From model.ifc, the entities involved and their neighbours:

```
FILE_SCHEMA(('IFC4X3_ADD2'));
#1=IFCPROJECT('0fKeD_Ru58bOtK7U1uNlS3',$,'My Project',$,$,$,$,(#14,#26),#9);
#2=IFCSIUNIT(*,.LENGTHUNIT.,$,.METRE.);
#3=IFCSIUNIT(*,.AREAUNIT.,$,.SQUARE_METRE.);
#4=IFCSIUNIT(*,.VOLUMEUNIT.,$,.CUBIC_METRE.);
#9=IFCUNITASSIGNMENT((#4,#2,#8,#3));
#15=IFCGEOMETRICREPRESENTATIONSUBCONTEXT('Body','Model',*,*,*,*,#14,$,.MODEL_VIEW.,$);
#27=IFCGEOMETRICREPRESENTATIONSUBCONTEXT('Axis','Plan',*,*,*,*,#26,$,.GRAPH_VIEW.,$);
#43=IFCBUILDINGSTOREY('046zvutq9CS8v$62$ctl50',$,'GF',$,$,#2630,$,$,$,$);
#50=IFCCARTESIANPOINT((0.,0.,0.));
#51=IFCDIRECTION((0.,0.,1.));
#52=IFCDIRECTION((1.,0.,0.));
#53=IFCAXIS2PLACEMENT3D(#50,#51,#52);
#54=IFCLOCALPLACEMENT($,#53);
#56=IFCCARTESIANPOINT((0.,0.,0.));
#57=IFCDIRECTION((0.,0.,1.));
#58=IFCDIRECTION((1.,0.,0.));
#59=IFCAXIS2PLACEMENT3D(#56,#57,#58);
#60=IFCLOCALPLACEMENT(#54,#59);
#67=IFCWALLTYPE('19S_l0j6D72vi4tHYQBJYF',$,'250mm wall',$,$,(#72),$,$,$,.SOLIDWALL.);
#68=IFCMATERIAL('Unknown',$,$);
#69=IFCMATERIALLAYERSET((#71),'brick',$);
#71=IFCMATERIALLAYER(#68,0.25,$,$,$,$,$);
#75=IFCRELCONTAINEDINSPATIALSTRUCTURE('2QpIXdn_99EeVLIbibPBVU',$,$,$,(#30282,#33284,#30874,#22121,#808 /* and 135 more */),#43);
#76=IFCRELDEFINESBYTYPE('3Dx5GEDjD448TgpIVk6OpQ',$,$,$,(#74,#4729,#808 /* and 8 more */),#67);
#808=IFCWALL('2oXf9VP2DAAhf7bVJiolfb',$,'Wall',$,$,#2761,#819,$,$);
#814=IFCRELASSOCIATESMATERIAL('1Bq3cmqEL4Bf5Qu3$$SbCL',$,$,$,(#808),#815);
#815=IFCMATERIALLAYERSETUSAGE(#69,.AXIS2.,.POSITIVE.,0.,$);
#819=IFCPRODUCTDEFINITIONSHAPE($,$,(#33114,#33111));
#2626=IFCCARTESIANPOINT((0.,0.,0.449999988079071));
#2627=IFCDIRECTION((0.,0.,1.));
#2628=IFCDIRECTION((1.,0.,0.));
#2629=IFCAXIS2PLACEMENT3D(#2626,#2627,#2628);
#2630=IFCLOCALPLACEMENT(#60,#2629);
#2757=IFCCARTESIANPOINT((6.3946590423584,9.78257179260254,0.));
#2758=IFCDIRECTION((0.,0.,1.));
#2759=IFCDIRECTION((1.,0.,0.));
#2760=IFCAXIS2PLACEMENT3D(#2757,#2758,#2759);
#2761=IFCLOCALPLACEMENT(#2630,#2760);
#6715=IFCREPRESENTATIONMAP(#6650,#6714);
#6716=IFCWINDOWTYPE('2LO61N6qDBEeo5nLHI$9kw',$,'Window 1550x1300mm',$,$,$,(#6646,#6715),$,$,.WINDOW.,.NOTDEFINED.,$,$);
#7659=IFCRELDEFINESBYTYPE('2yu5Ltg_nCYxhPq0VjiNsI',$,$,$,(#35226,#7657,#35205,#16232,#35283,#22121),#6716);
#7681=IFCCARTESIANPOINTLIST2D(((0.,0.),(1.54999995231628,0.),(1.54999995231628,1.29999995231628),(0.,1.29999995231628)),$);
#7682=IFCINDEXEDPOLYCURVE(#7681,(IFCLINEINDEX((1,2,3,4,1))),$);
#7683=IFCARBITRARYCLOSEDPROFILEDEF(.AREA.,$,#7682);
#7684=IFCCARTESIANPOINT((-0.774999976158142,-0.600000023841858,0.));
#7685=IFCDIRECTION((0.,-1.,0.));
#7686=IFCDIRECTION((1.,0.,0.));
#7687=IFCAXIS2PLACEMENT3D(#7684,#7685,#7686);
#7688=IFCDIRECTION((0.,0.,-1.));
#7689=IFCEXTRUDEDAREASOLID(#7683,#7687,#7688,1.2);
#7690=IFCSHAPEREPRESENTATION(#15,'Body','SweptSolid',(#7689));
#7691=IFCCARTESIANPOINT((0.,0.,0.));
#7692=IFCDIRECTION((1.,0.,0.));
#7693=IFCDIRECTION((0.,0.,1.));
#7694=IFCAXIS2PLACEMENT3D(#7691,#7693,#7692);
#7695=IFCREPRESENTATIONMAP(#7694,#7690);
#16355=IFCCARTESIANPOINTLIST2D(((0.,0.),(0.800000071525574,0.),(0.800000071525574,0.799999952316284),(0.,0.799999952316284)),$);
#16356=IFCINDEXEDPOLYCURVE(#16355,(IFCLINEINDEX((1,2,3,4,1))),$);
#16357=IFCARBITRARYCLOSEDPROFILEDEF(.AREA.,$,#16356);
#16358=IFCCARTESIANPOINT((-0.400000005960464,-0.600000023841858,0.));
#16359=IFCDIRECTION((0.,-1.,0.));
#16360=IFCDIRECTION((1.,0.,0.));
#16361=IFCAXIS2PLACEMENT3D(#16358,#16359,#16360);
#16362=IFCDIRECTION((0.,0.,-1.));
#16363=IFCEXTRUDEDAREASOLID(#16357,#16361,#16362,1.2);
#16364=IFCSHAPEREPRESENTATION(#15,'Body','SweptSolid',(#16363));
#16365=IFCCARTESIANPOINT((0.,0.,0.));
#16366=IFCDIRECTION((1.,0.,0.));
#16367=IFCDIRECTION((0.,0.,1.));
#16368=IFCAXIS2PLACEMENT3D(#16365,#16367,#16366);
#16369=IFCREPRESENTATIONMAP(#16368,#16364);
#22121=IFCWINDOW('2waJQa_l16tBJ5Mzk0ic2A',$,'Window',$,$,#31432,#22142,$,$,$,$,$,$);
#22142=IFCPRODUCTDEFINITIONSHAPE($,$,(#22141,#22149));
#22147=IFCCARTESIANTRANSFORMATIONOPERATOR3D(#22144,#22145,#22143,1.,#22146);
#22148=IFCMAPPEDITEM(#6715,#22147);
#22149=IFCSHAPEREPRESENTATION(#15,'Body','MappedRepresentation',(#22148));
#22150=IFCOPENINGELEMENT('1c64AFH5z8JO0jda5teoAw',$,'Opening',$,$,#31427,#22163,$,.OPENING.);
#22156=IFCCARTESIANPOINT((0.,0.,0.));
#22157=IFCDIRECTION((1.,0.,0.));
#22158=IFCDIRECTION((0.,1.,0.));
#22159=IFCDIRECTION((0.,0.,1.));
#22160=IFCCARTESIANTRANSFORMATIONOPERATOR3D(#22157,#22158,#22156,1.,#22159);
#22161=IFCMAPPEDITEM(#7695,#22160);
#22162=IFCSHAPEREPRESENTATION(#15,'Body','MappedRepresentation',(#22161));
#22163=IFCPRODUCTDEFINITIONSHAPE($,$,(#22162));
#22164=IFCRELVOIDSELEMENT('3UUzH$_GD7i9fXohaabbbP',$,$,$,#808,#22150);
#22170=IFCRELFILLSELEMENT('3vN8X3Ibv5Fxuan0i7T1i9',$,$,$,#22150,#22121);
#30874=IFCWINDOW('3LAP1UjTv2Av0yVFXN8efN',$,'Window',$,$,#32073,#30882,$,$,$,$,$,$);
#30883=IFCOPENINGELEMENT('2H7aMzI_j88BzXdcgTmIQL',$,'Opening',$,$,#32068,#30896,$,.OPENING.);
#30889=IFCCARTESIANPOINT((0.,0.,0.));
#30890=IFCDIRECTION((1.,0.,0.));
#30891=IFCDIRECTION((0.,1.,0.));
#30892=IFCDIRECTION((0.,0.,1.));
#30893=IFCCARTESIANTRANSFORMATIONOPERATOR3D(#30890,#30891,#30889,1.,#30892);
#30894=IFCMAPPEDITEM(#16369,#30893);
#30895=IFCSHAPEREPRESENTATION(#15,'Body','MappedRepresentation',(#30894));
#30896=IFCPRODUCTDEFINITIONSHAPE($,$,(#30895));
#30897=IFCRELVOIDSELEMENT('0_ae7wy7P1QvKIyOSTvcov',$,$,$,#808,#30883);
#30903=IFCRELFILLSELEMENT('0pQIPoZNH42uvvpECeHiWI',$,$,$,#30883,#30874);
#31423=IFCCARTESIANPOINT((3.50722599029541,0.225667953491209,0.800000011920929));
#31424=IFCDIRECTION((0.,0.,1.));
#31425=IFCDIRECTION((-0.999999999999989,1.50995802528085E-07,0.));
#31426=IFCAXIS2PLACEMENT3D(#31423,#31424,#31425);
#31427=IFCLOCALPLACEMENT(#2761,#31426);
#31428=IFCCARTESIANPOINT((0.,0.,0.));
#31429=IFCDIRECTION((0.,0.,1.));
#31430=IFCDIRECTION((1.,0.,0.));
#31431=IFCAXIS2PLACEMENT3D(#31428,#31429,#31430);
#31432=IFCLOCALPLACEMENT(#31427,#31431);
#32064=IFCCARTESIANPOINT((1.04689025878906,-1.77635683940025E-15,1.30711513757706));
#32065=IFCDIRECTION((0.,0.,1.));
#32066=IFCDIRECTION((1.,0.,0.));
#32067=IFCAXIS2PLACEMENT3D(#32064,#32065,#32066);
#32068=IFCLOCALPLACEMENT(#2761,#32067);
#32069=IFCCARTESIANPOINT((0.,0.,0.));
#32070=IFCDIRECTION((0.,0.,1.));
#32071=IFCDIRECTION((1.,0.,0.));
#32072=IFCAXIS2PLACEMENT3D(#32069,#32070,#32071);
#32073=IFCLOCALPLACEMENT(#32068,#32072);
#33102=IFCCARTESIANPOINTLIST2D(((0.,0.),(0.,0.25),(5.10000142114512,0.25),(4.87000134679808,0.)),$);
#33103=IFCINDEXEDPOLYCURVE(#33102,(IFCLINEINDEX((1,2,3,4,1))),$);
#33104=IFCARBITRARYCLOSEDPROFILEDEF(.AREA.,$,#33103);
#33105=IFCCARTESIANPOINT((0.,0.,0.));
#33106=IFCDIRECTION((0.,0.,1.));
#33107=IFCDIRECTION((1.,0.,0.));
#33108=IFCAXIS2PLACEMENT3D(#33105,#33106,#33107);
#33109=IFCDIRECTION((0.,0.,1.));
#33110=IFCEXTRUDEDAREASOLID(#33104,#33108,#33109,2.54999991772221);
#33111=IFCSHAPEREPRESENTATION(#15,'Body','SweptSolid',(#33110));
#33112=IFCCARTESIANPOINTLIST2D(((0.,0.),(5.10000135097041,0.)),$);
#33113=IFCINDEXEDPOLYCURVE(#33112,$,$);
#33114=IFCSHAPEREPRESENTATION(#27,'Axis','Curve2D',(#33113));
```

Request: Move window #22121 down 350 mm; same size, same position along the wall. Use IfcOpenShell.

```python
import numpy as np
import ifcopenshell
import ifcopenshell.api.geometry
import ifcopenshell.util.placement
import ifcopenshell.util.unit

model = ifcopenshell.open("model.ifc")
unit_scale = ifcopenshell.util.unit.calculate_unit_scale(model)

window = model.by_guid("2waJQa_l16tBJ5Mzk0ic2A")
opening = window.FillsVoids[0].RelatingOpeningElement
dz = -0.35 / unit_scale

shift = np.array([0.0, 0.0, dz])
# The window is placed relative to its opening, so it follows when the opening moves.
matrix = ifcopenshell.util.placement.get_local_placement(opening.ObjectPlacement)
matrix[:3, 3] += shift
ifcopenshell.api.geometry.edit_object_placement(
    model, product=opening, matrix=matrix, is_si=False, should_transform_children=True
)

print(f"moved by {dz * unit_scale:+.3f} m")

model.write("model_rev.ifc")
```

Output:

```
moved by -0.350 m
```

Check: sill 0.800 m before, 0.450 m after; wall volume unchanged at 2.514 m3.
